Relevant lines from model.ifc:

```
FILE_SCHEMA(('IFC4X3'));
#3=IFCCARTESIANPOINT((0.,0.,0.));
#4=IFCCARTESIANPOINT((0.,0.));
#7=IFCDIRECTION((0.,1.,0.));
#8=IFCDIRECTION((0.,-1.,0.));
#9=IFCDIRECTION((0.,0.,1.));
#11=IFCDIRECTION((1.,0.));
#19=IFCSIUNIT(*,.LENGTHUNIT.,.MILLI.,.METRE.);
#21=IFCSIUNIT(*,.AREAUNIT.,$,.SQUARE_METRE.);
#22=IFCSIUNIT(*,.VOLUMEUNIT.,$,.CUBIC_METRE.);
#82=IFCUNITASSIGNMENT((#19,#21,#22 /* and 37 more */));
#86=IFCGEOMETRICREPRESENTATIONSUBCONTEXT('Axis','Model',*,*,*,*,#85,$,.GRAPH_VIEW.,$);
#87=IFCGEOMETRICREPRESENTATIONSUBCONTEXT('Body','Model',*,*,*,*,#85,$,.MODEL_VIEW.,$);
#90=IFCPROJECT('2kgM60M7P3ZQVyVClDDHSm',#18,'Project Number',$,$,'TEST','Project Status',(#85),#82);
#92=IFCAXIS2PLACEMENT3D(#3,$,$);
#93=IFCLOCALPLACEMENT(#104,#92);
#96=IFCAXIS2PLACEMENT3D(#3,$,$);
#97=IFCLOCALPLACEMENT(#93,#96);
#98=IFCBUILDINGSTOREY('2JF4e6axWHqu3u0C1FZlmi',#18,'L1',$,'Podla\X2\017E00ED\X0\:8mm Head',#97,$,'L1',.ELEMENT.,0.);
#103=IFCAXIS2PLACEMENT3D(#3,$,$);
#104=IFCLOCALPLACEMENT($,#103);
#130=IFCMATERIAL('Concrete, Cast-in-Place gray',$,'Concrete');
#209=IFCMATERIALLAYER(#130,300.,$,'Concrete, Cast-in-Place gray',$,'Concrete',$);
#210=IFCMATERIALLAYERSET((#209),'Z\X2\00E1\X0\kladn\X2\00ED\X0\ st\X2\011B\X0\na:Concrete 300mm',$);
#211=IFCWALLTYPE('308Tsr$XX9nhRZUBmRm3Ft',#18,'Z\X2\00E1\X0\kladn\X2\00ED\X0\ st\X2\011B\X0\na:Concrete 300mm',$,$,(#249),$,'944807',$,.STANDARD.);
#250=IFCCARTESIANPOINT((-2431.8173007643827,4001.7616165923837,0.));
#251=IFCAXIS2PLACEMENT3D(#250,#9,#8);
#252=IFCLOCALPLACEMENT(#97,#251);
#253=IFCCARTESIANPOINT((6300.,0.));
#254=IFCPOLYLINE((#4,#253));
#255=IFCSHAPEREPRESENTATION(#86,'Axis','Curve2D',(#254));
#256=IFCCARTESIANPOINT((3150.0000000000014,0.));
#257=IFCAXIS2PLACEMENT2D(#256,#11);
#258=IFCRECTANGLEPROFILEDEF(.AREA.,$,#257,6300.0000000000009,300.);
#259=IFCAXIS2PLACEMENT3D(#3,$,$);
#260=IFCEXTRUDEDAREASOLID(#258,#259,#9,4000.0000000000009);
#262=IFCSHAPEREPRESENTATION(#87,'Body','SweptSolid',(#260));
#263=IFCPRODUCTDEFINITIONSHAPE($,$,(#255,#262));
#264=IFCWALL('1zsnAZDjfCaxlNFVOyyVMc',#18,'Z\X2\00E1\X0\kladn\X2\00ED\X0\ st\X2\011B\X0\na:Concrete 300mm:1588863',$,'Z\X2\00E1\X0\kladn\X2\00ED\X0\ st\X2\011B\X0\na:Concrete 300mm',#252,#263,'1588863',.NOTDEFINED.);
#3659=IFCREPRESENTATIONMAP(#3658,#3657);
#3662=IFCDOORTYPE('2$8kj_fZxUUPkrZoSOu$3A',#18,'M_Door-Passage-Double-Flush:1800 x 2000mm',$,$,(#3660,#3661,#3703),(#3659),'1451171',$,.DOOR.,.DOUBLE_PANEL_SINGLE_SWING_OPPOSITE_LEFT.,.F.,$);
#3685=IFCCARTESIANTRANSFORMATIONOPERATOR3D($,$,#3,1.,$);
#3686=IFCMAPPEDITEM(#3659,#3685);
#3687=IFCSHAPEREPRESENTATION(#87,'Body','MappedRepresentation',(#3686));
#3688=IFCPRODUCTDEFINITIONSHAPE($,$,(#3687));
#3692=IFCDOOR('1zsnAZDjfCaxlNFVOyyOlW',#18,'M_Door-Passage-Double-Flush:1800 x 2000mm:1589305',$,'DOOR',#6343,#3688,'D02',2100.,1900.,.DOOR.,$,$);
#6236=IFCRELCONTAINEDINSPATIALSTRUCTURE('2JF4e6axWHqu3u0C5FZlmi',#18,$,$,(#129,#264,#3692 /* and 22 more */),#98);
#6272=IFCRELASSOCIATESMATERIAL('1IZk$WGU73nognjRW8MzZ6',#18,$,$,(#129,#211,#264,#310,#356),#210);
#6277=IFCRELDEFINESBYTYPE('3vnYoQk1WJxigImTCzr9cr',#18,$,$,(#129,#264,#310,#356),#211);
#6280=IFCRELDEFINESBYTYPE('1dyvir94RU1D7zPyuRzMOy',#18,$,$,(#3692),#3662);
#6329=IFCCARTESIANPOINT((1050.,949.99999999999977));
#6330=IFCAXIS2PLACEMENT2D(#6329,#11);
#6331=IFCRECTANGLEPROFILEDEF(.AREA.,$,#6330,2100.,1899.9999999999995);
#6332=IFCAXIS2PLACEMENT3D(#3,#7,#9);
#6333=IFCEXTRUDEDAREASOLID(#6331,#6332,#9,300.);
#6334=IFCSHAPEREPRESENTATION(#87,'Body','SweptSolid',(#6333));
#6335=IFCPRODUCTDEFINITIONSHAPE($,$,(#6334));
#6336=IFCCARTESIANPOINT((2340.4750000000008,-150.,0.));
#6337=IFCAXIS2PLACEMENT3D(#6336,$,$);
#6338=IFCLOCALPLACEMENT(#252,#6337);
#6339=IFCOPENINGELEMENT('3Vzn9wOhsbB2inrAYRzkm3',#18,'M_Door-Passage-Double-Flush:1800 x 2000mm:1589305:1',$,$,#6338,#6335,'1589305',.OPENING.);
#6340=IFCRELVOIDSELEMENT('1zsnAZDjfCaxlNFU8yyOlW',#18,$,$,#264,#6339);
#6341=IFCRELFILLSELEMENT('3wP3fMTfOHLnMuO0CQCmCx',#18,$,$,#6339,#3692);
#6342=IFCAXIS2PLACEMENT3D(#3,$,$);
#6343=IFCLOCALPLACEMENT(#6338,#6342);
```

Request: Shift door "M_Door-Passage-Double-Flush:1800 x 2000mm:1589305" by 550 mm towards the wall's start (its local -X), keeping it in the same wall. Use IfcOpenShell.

```python
import ifcopenshell
import ifcopenshell.api.geometry
import ifcopenshell.util.placement
import ifcopenshell.util.unit

model = ifcopenshell.open("model.ifc")
unit_scale = ifcopenshell.util.unit.calculate_unit_scale(model)

door = model.by_id(3692)
opening = door.FillsVoids[0].RelatingOpeningElement
wall = opening.VoidsElements[0].RelatingBuildingElement

wall_matrix = ifcopenshell.util.placement.get_local_placement(wall.ObjectPlacement)
shift = wall_matrix[:3, 0] * -0.55 / unit_scale
before = ifcopenshell.util.placement.get_local_placement(door.ObjectPlacement)[:3, 3].copy()

# The door is placed relative to its opening, so it follows when the opening moves.
matrix = ifcopenshell.util.placement.get_local_placement(opening.ObjectPlacement)
matrix[:3, 3] += shift
ifcopenshell.api.geometry.edit_object_placement(
    model, product=opening, matrix=matrix, is_si=False, should_transform_children=True
)

after = ifcopenshell.util.placement.get_local_placement(door.ObjectPlacement)[:3, 3]
print("door moved by", (after - before).round(3) + 0.0)

model.write("model_updated.ifc")
```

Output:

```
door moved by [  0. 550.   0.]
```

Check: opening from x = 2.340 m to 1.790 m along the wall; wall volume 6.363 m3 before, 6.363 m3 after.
